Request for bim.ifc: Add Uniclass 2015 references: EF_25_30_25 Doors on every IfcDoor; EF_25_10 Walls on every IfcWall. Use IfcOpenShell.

First a look at what the model holds.

```python
import ifcopenshell

model = ifcopenshell.open("bim.ifc")
print(model.schema)
print("classifications:", [c.Name for c in model.by_type("IfcClassification")])
for ifc_class in ("IfcDoor", "IfcRoof", "IfcStair", "IfcWall", "IfcWindow"):
    print(ifc_class, len(model.by_type(ifc_class)))
```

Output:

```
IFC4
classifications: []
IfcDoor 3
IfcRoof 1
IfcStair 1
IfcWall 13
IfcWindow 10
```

```python
import ifcopenshell
import ifcopenshell.api.classification

model = ifcopenshell.open("bim.ifc")

system = ifcopenshell.api.classification.add_classification(model, classification="Uniclass 2015")

codes = {
    "IfcDoor": ("EF_25_30_25", "Doors"),
    "IfcWall": ("EF_25_10", "Walls"),
}
for ifc_class, (code, name) in codes.items():
    products = model.by_type(ifc_class)
    ifcopenshell.api.classification.add_reference(
        model, products=products, classification=system, identification=code, name=name
    )
    print(code, len(products))

model.write("bim_updated.ifc")
```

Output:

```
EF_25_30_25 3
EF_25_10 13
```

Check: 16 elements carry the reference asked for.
